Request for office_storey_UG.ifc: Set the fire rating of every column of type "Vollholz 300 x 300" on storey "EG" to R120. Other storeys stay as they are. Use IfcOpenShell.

First a look at what the model holds.

```python
import ifcopenshell
import ifcopenshell.util.element

model = ifcopenshell.open("office_storey_UG.ifc")
print(model.schema)
storey = next(s for s in model.by_type("IfcBuildingStorey") if s.Name == "EG")
columns = [e for e in ifcopenshell.util.element.get_decomposition(storey) if e.is_a("IfcColumn")]
seen = {}
for e in columns:
    element_type = ifcopenshell.util.element.get_type(e)
    key = (element_type.Name if element_type != e and element_type else None, ifcopenshell.util.element.get_pset(e, "Pset_ColumnCommon", "FireRating"))
    seen[key] = seen.get(key, 0) + 1
for (name, value), count in sorted(seen.items(), key=str):
    print(count, "x", name, "|", value)
```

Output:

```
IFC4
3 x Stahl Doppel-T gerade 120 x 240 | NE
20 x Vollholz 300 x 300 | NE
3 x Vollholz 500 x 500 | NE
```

```python
import ifcopenshell
import ifcopenshell.api.pset
import ifcopenshell.util.element

model = ifcopenshell.open("office_storey_UG.ifc")

storey = next(s for s in model.by_type("IfcBuildingStorey") if s.Name == "EG")
columns = [e for e in ifcopenshell.util.element.get_decomposition(storey) if e.is_a("IfcColumn")]

count = 0
for e in columns:
    element_type = ifcopenshell.util.element.get_type(e)
    if element_type in (None, e) or element_type.Name != "Vollholz 300 x 300":
        continue
    # add_pset returns the element's existing set when there is one.
    pset = ifcopenshell.api.pset.add_pset(model, product=e, name="Pset_ColumnCommon")
    ifcopenshell.api.pset.edit_pset(model, pset=pset, properties={"FireRating": "R120"})
    count += 1

print(count, "columns updated")

model.write("office_storey_UG_updated.ifc")
```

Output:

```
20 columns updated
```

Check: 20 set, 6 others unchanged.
